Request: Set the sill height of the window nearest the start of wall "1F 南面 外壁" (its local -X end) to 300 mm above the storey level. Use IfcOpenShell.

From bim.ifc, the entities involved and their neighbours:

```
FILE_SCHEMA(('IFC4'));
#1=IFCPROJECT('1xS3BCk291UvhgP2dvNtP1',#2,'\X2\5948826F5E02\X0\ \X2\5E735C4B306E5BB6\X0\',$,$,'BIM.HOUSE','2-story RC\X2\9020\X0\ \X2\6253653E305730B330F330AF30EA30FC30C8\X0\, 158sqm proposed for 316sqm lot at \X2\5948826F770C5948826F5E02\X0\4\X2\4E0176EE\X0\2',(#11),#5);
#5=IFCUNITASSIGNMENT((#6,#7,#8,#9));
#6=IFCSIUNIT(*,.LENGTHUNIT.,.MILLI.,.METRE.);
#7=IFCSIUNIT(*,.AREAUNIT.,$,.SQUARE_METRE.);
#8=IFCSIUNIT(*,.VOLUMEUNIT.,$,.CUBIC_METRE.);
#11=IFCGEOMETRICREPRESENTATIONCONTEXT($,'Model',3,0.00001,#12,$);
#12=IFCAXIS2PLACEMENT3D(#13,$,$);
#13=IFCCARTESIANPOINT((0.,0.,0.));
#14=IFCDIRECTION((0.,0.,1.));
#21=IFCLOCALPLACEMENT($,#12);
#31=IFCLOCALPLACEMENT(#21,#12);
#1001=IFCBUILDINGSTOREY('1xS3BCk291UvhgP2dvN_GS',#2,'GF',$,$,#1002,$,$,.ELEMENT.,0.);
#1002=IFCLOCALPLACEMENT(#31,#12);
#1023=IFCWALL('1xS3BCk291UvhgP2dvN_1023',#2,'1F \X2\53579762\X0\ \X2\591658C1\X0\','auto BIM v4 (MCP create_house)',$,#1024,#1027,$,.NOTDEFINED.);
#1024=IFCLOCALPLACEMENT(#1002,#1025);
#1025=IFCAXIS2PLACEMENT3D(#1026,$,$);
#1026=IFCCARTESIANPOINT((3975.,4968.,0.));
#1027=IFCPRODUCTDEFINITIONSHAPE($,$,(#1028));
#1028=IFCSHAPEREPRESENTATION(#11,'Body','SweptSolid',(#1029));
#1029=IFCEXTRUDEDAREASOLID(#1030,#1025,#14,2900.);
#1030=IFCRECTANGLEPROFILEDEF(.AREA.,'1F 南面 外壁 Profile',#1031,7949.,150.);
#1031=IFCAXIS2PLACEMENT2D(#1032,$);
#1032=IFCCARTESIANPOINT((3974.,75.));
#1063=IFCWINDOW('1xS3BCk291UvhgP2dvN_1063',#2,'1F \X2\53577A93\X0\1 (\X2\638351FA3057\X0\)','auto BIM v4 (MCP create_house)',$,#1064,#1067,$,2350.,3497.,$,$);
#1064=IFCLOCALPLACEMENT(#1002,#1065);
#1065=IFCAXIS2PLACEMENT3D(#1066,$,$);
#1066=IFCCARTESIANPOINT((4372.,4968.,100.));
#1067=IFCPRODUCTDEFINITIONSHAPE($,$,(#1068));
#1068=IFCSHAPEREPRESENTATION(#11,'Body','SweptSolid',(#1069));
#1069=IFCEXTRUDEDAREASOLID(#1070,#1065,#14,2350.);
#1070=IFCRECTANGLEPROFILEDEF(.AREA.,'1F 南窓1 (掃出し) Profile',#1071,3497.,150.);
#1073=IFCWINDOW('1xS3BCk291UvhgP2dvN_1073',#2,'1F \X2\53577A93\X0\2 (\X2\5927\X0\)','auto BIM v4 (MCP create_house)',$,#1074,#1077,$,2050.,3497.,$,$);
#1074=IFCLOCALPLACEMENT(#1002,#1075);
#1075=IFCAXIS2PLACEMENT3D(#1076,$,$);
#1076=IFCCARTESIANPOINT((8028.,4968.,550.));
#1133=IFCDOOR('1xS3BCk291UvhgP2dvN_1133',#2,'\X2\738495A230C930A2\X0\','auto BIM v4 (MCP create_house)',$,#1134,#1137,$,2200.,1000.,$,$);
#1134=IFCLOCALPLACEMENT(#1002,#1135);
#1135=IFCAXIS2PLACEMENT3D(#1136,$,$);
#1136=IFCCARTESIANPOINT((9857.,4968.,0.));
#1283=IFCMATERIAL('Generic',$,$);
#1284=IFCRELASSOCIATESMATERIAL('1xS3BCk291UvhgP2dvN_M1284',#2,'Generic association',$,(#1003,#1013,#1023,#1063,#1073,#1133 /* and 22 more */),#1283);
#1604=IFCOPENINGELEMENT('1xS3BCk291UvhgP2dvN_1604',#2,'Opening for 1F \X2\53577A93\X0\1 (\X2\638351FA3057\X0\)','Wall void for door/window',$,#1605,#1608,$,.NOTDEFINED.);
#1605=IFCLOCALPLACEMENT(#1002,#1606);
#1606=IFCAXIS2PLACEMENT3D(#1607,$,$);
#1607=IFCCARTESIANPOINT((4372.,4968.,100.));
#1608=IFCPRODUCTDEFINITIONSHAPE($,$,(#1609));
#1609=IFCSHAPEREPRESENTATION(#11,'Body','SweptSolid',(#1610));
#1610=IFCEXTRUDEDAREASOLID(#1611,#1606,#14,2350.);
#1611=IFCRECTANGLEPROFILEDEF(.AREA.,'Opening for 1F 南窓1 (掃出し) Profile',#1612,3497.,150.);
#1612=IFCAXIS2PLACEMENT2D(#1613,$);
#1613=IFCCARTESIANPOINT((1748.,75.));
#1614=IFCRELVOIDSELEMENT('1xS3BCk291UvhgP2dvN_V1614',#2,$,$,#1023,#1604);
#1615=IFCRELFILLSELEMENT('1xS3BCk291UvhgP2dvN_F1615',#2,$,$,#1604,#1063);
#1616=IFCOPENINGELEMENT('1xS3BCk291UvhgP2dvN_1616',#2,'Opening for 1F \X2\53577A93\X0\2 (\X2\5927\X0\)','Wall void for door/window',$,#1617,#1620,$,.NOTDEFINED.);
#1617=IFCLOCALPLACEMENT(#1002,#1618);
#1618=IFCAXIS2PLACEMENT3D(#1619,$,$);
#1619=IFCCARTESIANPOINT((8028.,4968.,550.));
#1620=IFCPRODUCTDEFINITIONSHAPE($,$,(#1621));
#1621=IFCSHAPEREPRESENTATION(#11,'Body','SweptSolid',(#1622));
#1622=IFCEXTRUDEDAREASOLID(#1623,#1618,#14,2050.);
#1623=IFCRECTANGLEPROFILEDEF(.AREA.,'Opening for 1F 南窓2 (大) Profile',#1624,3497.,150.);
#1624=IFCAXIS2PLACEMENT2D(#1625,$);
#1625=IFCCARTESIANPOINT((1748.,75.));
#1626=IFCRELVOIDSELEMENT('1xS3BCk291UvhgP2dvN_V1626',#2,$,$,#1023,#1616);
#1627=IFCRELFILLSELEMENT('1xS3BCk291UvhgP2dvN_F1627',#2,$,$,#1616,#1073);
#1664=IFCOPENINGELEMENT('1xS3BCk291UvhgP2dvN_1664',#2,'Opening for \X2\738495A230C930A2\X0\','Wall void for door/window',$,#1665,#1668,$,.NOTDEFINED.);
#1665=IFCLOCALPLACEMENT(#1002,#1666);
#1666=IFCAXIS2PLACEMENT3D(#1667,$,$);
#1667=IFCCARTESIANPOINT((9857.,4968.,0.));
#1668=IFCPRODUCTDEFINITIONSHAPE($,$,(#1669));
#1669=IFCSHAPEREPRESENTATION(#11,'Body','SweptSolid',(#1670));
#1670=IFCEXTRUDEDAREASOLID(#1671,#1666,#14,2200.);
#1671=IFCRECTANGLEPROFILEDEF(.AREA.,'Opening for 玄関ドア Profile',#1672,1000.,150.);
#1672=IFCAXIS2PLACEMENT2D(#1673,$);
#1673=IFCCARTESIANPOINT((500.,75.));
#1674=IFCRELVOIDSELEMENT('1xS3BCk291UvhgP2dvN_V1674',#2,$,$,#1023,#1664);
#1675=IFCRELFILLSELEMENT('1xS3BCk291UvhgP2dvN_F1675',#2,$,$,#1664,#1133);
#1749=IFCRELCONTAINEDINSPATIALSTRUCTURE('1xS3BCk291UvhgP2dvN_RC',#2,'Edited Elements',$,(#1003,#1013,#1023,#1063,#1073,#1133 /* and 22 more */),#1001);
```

```python
import numpy as np
import ifcopenshell
import ifcopenshell.api.geometry
import ifcopenshell.geom
import ifcopenshell.util.element
import ifcopenshell.util.placement
import ifcopenshell.util.shape
import ifcopenshell.util.unit

model = ifcopenshell.open("bim.ifc")
unit_scale = ifcopenshell.util.unit.calculate_unit_scale(model)

window = model.by_id(1063)
opening = window.FillsVoids[0].RelatingOpeningElement
storey = ifcopenshell.util.element.get_container(window, ifc_class="IfcBuildingStorey")
level = ifcopenshell.util.placement.get_local_placement(storey.ObjectPlacement)[2, 3]

# The opening's origin need not be at the sill, so measure its lowest point.
shape = ifcopenshell.geom.create_shape(ifcopenshell.geom.settings(), opening)
bottom = ifcopenshell.util.shape.get_shape_bottom_elevation(shape, shape.geometry) / unit_scale
dz = level + 0.3 / unit_scale - bottom

shift = np.array([0.0, 0.0, dz])
# The window is not placed relative to its opening, so move both.
for product in (opening, window):
    matrix = ifcopenshell.util.placement.get_local_placement(product.ObjectPlacement)
    matrix[:3, 3] += shift
    ifcopenshell.api.geometry.edit_object_placement(model, product=product, matrix=matrix, is_si=False)

print(f"moved by {dz * unit_scale:+.3f} m")

model.write("bim-out.ifc")
```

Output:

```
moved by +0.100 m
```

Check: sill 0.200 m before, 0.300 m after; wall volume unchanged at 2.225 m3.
